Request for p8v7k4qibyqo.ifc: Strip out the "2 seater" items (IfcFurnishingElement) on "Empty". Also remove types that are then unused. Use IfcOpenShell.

First a look at what the model holds.

```python
import ifcopenshell
import ifcopenshell.util.element

model = ifcopenshell.open("p8v7k4qibyqo.ifc")
print(model.schema)
storey = next(s for s in model.by_type("IfcBuildingStorey") if s.Name == "Empty")
furniture = [e for e in ifcopenshell.util.element.get_decomposition(storey) if e.is_a("IfcFurnishingElement")]
seen = {}
for e in furniture:
    element_type = ifcopenshell.util.element.get_type(e)
    name = element_type.Name if element_type not in (None, e) else None
    seen[name] = seen.get(name, 0) + 1
for name, count in sorted(seen.items(), key=str):
    print(count, "x", name)
```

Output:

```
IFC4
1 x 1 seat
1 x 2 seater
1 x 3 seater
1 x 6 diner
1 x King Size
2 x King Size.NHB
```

```python
import ifcopenshell
import ifcopenshell.api.root
import ifcopenshell.util.element

model = ifcopenshell.open("p8v7k4qibyqo.ifc")

storey = next(s for s in model.by_type("IfcBuildingStorey") if s.Name == "Empty")
furniture = [e for e in ifcopenshell.util.element.get_decomposition(storey) if e.is_a("IfcFurnishingElement")]
targets = [e for e in furniture if (t := ifcopenshell.util.element.get_type(e)) not in (None, e) and t.Name == "2 seater"]
types = {ifcopenshell.util.element.get_type(e) for e in targets} - {None, *targets}

for e in targets:
    ifcopenshell.api.root.remove_product(model, product=e)
print(len(targets), "removed")

unused = [t for t in types if not ifcopenshell.util.element.get_types(t)]
for t in unused:
    ifcopenshell.api.root.remove_product(model, product=t)
print(len(unused), "unused types removed")

model.write("p8v7k4qibyqo-out.ifc")
```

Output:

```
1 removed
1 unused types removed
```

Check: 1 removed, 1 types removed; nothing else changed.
